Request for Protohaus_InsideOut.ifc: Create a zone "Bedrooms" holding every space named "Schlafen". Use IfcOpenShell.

First a look at what the model holds.

```python
import ifcopenshell

model = ifcopenshell.open("Protohaus_InsideOut.ifc")
print(model.schema)
seen = {}
for space in model.by_type("IfcSpace"):
    seen[space.LongName] = seen.get(space.LongName, 0) + 1
for name, count in sorted(seen.items(), key=str):
    print(count, "x", name)
print("zones:", [z.Name for z in model.by_type("IfcZone")][:20])
```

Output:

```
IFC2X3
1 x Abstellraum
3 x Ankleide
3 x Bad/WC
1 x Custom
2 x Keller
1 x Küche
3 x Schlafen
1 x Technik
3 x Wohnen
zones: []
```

```python
import ifcopenshell
import ifcopenshell.api.group
import ifcopenshell.api.root

model = ifcopenshell.open("Protohaus_InsideOut.ifc")

names = {"Schlafen"}
spaces = [s for s in model.by_type("IfcSpace") if s.LongName in names]

zone = ifcopenshell.api.root.create_entity(model, ifc_class="IfcZone", name="Bedrooms")
ifcopenshell.api.group.assign_group(model, products=spaces, group=zone)
print(len(spaces), "spaces in", zone.Name)

model.write("Protohaus_InsideOut_rev.ifc")
```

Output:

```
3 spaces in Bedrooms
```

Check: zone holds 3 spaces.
